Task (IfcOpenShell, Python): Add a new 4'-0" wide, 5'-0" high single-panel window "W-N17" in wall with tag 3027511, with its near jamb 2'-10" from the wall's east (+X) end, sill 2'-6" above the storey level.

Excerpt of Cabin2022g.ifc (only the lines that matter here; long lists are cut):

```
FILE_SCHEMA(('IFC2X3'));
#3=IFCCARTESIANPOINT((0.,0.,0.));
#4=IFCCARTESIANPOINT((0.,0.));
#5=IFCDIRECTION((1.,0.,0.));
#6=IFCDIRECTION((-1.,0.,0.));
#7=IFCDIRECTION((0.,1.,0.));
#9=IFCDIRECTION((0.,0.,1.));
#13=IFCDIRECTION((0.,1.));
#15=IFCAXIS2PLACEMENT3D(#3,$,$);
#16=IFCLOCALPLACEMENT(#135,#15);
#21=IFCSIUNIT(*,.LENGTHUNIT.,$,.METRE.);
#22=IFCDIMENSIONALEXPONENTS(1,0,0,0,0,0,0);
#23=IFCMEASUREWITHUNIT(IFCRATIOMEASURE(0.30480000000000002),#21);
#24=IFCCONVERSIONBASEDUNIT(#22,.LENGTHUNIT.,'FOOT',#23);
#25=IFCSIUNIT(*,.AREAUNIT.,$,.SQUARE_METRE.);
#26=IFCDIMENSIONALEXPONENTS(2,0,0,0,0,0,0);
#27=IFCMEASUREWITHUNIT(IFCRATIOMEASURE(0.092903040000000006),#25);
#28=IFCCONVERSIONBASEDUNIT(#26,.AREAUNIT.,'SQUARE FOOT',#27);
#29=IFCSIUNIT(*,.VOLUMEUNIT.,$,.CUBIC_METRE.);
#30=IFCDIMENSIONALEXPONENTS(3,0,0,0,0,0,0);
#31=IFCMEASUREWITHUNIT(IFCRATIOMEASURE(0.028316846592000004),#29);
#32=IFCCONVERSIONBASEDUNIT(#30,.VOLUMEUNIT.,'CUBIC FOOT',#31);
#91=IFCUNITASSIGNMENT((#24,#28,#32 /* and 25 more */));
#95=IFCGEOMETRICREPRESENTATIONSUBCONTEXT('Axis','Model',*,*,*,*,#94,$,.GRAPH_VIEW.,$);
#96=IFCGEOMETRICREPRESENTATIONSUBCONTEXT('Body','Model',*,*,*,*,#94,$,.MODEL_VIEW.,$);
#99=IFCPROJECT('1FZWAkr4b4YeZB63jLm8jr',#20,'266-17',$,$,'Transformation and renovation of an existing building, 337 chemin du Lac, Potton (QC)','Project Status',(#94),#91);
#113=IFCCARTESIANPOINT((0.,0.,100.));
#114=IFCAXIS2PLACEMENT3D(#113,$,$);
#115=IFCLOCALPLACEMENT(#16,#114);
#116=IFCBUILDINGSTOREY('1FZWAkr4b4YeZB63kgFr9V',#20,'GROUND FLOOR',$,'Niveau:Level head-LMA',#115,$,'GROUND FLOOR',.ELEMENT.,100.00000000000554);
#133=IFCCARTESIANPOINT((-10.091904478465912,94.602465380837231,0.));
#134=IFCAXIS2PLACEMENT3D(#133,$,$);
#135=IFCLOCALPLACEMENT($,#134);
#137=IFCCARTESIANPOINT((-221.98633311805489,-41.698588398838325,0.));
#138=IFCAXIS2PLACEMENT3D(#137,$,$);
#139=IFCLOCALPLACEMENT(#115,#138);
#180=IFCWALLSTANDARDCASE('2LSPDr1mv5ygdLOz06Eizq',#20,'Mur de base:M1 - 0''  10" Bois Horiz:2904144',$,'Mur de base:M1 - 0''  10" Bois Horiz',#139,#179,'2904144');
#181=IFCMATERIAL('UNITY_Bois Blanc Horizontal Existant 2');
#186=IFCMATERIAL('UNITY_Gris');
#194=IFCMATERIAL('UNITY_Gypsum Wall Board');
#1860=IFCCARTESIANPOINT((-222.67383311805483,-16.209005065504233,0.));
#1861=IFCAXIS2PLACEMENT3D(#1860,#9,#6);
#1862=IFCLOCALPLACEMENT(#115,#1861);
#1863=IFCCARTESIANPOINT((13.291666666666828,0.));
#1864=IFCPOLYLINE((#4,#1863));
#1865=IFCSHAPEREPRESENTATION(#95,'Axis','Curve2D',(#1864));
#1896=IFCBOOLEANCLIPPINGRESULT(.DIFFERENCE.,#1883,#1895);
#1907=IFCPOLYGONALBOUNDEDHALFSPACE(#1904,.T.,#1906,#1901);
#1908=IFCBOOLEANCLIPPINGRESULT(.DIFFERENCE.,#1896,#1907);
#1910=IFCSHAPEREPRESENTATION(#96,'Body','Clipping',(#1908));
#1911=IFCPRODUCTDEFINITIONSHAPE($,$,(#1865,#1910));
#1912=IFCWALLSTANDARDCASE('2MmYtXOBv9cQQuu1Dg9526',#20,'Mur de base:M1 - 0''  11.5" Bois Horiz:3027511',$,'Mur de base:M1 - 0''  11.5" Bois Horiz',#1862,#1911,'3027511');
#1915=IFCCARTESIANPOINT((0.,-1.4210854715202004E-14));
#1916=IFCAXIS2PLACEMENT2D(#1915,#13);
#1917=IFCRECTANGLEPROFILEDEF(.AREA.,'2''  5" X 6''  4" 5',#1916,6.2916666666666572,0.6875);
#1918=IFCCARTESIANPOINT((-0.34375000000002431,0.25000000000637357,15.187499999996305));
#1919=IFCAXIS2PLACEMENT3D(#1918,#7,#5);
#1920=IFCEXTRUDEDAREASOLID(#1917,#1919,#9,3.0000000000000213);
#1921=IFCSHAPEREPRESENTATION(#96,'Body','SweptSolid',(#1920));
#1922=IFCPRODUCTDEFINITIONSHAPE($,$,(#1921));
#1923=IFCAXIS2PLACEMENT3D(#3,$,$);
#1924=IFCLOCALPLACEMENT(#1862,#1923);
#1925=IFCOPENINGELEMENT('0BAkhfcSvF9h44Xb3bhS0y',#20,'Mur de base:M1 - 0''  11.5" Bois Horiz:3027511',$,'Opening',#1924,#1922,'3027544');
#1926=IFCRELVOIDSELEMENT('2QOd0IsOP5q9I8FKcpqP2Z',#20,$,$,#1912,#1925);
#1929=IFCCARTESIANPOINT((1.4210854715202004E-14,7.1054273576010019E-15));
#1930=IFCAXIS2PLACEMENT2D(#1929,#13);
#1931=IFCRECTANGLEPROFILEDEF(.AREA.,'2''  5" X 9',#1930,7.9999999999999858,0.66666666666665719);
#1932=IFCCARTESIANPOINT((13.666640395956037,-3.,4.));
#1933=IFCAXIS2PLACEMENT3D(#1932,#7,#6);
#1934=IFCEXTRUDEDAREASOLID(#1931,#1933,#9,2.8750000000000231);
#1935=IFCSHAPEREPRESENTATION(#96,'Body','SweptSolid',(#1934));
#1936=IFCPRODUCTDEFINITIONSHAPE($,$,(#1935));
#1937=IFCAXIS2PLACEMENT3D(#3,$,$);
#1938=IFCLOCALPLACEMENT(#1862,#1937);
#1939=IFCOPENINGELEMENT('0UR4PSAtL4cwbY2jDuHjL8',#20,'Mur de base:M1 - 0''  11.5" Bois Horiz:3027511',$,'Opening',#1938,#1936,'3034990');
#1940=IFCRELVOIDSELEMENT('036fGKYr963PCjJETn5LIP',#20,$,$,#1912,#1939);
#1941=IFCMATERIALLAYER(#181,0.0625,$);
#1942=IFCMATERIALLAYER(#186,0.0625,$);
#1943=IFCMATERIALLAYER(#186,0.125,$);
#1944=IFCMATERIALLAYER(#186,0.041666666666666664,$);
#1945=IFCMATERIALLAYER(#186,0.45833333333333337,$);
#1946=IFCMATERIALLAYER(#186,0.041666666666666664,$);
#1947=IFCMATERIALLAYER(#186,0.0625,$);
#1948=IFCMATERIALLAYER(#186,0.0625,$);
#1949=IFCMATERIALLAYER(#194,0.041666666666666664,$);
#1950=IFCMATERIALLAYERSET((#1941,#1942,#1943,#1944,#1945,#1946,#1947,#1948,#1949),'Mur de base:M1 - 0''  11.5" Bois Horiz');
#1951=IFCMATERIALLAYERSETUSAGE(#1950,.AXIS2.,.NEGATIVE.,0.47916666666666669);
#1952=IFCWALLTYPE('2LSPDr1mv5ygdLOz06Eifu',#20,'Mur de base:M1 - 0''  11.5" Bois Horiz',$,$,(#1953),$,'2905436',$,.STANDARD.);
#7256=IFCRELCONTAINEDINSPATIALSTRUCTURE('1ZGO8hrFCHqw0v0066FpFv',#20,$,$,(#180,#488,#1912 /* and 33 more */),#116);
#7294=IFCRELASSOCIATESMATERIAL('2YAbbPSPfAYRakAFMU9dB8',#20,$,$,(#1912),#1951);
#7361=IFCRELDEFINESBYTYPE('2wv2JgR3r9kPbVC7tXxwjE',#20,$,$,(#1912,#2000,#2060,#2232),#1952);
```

```python
import numpy as np
import ifcopenshell
import ifcopenshell.api.feature
import ifcopenshell.api.geometry
import ifcopenshell.api.root
import ifcopenshell.api.spatial
import ifcopenshell.api.type
import ifcopenshell.geom
import ifcopenshell.util.element
import ifcopenshell.util.placement
import ifcopenshell.util.representation
import ifcopenshell.util.shape
import ifcopenshell.util.unit

model = ifcopenshell.open("Cabin2022g.ifc")
unit_scale = ifcopenshell.util.unit.calculate_unit_scale(model)
settings = ifcopenshell.geom.settings()


def volume(element):
    """Net volume in cubic metres, openings subtracted."""
    shape = ifcopenshell.geom.create_shape(settings, element)
    return ifcopenshell.util.shape.get_volume(shape.geometry)


wall = model.by_guid("2MmYtXOBv9cQQuu1Dg9526")
storey = ifcopenshell.util.element.get_container(wall, ifc_class="IfcBuildingStorey")
context = ifcopenshell.util.representation.get_context(model, "Model", "Body", "MODEL_VIEW")
before = volume(wall)

width, height, from_end, sill = 1.2192, 1.524, 0.8636, 0.762  # metres

# The wall runs along its own X axis, and the end named is its -X end.
wall_shape = ifcopenshell.geom.create_shape(settings, wall)
x, y, z = ifcopenshell.util.shape.get_vertices(wall_shape.geometry).T
start = x.min() + from_end
face, thickness = float(y.min()), float(y.max() - y.min())
wall_matrix = ifcopenshell.util.placement.get_local_placement(wall.ObjectPlacement)
level = ifcopenshell.util.placement.get_local_placement(storey.ObjectPlacement)[2, 3]


def in_wall(x, y):
    """Placement at x, y metres in the wall's axes, at sill height."""
    matrix = wall_matrix.copy()
    matrix[:, 3] = wall_matrix @ np.array([x / unit_scale, y / unit_scale, 0.0, 1.0])
    matrix[2, 3] = level + sill / unit_scale
    return matrix


# Opening: a box that overshoots both wall faces by 50 mm.
opening = ifcopenshell.api.root.create_entity(model, ifc_class="IfcOpeningElement")
box = ifcopenshell.api.geometry.add_wall_representation(
    model, context=context, length=width, height=height, thickness=thickness + 0.1
)
ifcopenshell.api.geometry.assign_representation(model, product=opening, representation=box)
ifcopenshell.api.geometry.edit_object_placement(model, product=opening, matrix=in_wall(start, face - 0.05), is_si=False)
ifcopenshell.api.feature.add_feature(model, feature=opening, element=wall)

window = ifcopenshell.api.root.create_entity(model, ifc_class="IfcWindow", name="W-N17")
window.OverallWidth, window.OverallHeight = width / unit_scale, height / unit_scale
body = ifcopenshell.api.geometry.add_window_representation(
    model,
    context=context,
    overall_width=window.OverallWidth,
    overall_height=window.OverallHeight,
    partition_type="SINGLE_PANEL",
)
ifcopenshell.api.geometry.assign_representation(model, product=window, representation=body)
ifcopenshell.api.spatial.assign_container(model, products=[window], relating_structure=storey)
fills = ifcopenshell.api.feature.add_filling(model, opening=opening, element=window)
fills.OwnerHistory = window.OwnerHistory  # required in IFC2X3

# IFC2X3 keeps the operation on the window style.
style = ifcopenshell.api.root.create_entity(model, ifc_class="IfcWindowStyle", name="W-N17")
style.OperationType, style.ConstructionType = "SINGLE_PANEL", "NOTDEFINED"
style.ParameterTakesPrecedence = style.Sizeable = False
ifcopenshell.api.type.assign_type(model, related_objects=[window], relating_type=style)

# Centre the window in the wall's thickness.
ifcopenshell.api.geometry.edit_object_placement(model, product=window, matrix=in_wall(start, face), is_si=False)
window_shape = ifcopenshell.geom.create_shape(settings, window)
depth = ifcopenshell.util.shape.get_vertices(window_shape.geometry)[:, 1]
offset = face + thickness / 2 - (depth.min() + depth.max()) / 2
ifcopenshell.api.geometry.edit_object_placement(model, product=window, matrix=in_wall(start, offset), is_si=False)

after = volume(wall)

print(f"wall volume {before:.3f} -> {after:.3f} m3")

model.write("Cabin2022g-out.ifc")
```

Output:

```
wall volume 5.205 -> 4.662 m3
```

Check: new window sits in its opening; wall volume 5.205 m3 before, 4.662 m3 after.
